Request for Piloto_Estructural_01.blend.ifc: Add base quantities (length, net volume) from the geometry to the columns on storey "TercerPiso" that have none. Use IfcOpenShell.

First a look at what the model holds.

```python
import ifcopenshell
import ifcopenshell.util.element
import ifcopenshell.util.unit

model = ifcopenshell.open("Piloto_Estructural_01.blend.ifc")
print(model.schema)
for unit_type in ("LENGTHUNIT", "AREAUNIT", "VOLUMEUNIT"):
    print(unit_type, ifcopenshell.util.unit.calculate_unit_scale(model, unit_type))
storey = next(s for s in model.by_type("IfcBuildingStorey") if s.Name == "TercerPiso")
columns = [e for e in ifcopenshell.util.element.get_decomposition(storey) if e.is_a("IfcColumn")]
for e in sorted(columns, key=lambda e: e.id()):
    print(e.id(), e.is_a(), e.Name, list(ifcopenshell.util.element.get_psets(e, qtos_only=True)), sep=" | ")
```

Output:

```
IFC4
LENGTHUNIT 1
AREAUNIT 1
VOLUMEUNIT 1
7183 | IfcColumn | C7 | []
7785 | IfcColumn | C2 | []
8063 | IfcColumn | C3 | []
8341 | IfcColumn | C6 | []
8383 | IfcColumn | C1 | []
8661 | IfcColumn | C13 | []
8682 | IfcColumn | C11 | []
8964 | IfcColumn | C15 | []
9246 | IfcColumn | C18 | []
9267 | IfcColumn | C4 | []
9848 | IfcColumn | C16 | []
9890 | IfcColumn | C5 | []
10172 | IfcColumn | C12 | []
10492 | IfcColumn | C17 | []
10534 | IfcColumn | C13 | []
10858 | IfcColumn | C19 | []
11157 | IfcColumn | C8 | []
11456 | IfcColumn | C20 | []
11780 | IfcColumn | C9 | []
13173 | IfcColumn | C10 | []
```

```python
import ifcopenshell
import ifcopenshell.api.pset
import ifcopenshell.geom
import ifcopenshell.util.element
import ifcopenshell.util.shape
import ifcopenshell.util.unit

model = ifcopenshell.open("Piloto_Estructural_01.blend.ifc")
unit_scale = ifcopenshell.util.unit.calculate_unit_scale(model)
volume_scale = ifcopenshell.util.unit.calculate_unit_scale(model, "VOLUMEUNIT")
settings = ifcopenshell.geom.settings()

storey = next(s for s in model.by_type("IfcBuildingStorey") if s.Name == "TercerPiso")
columns = [e for e in ifcopenshell.util.element.get_decomposition(storey) if e.is_a("IfcColumn")]

for e in sorted(columns, key=lambda e: e.id()):
    if ifcopenshell.util.element.get_psets(e, qtos_only=True, should_inherit=False):
        continue
    # Geometry comes back in metres, in the element's own axes.
    shape = ifcopenshell.geom.create_shape(settings, e)
    values = {
        "Length": ifcopenshell.util.shape.get_z(shape.geometry) / unit_scale,
        "NetVolume": ifcopenshell.util.shape.get_volume(shape.geometry) / volume_scale,
    }
    qto = ifcopenshell.api.pset.add_qto(model, product=e, name="Qto_ColumnBaseQuantities")
    ifcopenshell.api.pset.edit_qto(model, qto=qto, properties=values)
    print(e.id(), {k: round(v, 3) for k, v in values.items()})

model.write("Piloto_Estructural_01.blend_rev.ifc")
```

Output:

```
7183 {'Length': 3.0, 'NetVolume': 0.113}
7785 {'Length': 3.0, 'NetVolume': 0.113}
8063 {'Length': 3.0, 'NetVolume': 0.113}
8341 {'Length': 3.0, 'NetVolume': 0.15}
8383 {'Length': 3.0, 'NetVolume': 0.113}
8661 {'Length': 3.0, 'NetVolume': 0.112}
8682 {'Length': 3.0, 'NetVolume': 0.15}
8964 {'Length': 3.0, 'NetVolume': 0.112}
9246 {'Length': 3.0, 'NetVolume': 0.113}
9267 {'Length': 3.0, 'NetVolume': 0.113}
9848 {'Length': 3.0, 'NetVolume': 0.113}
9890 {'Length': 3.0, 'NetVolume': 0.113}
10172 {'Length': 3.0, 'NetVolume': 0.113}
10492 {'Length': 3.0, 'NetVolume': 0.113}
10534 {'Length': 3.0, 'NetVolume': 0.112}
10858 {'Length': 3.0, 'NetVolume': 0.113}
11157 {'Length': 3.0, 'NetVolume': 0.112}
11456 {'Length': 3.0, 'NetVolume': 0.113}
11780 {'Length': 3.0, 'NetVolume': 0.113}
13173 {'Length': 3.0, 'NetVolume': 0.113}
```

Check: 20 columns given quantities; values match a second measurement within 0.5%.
